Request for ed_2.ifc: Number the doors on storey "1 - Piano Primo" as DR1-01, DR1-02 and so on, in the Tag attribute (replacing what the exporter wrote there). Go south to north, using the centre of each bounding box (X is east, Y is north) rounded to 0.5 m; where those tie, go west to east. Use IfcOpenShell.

First a look at what the model holds.

```python
import ifcopenshell
import ifcopenshell.util.element
import ifcopenshell.util.placement

model = ifcopenshell.open("ed_2.ifc")
print(model.schema)
storey = next(s for s in model.by_type("IfcBuildingStorey") if s.Name == "1 - Piano Primo")
doors = [e for e in ifcopenshell.util.element.get_decomposition(storey) if e.is_a("IfcDoor")]
for e in sorted(doors, key=lambda e: e.id()):
    origin = ifcopenshell.util.placement.get_local_placement(e.ObjectPlacement)[:3, 3]
    print(e.id(), e.Tag, e.Name, origin.round(2) + 0.0, sep=" | ")
```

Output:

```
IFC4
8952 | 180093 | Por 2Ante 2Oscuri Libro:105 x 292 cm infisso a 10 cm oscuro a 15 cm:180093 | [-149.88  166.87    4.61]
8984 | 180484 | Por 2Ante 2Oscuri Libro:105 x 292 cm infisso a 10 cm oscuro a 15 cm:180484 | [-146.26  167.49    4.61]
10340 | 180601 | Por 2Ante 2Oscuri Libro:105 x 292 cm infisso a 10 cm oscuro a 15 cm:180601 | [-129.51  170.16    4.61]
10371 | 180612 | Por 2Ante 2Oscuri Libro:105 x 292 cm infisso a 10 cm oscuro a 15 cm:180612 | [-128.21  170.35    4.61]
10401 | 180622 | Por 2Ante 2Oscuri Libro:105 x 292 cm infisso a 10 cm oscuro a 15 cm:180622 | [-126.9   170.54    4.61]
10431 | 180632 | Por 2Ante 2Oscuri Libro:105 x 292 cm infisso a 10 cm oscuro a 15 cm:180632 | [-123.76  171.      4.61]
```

```python
import ifcopenshell
import ifcopenshell.geom
import ifcopenshell.util.element
import ifcopenshell.util.shape

model = ifcopenshell.open("ed_2.ifc")
settings = ifcopenshell.geom.settings()
settings.set("use-world-coords", True)


def centre(element):
    shape = ifcopenshell.geom.create_shape(settings, element)
    return ifcopenshell.util.shape.get_bbox_centroid(shape.geometry)


storey = next(s for s in model.by_type("IfcBuildingStorey") if s.Name == "1 - Piano Primo")
doors = [e for e in ifcopenshell.util.element.get_decomposition(storey) if e.is_a("IfcDoor")]

# Insertion points can sit at a corner or the storey origin, so sort by the geometry (in metres).
centres = {e: centre(e) for e in doors}
doors.sort(key=lambda e: (round(centres[e][1] / 0.5), centres[e][0]))

for i, e in enumerate(doors, start=1):
    number = f"DR1-{i:02d}"
    e.Tag = number
    print(e.id(), number)

model.write("ed_2_rev.ifc")
```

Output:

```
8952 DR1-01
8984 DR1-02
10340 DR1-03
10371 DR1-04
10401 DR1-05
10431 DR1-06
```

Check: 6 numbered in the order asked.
